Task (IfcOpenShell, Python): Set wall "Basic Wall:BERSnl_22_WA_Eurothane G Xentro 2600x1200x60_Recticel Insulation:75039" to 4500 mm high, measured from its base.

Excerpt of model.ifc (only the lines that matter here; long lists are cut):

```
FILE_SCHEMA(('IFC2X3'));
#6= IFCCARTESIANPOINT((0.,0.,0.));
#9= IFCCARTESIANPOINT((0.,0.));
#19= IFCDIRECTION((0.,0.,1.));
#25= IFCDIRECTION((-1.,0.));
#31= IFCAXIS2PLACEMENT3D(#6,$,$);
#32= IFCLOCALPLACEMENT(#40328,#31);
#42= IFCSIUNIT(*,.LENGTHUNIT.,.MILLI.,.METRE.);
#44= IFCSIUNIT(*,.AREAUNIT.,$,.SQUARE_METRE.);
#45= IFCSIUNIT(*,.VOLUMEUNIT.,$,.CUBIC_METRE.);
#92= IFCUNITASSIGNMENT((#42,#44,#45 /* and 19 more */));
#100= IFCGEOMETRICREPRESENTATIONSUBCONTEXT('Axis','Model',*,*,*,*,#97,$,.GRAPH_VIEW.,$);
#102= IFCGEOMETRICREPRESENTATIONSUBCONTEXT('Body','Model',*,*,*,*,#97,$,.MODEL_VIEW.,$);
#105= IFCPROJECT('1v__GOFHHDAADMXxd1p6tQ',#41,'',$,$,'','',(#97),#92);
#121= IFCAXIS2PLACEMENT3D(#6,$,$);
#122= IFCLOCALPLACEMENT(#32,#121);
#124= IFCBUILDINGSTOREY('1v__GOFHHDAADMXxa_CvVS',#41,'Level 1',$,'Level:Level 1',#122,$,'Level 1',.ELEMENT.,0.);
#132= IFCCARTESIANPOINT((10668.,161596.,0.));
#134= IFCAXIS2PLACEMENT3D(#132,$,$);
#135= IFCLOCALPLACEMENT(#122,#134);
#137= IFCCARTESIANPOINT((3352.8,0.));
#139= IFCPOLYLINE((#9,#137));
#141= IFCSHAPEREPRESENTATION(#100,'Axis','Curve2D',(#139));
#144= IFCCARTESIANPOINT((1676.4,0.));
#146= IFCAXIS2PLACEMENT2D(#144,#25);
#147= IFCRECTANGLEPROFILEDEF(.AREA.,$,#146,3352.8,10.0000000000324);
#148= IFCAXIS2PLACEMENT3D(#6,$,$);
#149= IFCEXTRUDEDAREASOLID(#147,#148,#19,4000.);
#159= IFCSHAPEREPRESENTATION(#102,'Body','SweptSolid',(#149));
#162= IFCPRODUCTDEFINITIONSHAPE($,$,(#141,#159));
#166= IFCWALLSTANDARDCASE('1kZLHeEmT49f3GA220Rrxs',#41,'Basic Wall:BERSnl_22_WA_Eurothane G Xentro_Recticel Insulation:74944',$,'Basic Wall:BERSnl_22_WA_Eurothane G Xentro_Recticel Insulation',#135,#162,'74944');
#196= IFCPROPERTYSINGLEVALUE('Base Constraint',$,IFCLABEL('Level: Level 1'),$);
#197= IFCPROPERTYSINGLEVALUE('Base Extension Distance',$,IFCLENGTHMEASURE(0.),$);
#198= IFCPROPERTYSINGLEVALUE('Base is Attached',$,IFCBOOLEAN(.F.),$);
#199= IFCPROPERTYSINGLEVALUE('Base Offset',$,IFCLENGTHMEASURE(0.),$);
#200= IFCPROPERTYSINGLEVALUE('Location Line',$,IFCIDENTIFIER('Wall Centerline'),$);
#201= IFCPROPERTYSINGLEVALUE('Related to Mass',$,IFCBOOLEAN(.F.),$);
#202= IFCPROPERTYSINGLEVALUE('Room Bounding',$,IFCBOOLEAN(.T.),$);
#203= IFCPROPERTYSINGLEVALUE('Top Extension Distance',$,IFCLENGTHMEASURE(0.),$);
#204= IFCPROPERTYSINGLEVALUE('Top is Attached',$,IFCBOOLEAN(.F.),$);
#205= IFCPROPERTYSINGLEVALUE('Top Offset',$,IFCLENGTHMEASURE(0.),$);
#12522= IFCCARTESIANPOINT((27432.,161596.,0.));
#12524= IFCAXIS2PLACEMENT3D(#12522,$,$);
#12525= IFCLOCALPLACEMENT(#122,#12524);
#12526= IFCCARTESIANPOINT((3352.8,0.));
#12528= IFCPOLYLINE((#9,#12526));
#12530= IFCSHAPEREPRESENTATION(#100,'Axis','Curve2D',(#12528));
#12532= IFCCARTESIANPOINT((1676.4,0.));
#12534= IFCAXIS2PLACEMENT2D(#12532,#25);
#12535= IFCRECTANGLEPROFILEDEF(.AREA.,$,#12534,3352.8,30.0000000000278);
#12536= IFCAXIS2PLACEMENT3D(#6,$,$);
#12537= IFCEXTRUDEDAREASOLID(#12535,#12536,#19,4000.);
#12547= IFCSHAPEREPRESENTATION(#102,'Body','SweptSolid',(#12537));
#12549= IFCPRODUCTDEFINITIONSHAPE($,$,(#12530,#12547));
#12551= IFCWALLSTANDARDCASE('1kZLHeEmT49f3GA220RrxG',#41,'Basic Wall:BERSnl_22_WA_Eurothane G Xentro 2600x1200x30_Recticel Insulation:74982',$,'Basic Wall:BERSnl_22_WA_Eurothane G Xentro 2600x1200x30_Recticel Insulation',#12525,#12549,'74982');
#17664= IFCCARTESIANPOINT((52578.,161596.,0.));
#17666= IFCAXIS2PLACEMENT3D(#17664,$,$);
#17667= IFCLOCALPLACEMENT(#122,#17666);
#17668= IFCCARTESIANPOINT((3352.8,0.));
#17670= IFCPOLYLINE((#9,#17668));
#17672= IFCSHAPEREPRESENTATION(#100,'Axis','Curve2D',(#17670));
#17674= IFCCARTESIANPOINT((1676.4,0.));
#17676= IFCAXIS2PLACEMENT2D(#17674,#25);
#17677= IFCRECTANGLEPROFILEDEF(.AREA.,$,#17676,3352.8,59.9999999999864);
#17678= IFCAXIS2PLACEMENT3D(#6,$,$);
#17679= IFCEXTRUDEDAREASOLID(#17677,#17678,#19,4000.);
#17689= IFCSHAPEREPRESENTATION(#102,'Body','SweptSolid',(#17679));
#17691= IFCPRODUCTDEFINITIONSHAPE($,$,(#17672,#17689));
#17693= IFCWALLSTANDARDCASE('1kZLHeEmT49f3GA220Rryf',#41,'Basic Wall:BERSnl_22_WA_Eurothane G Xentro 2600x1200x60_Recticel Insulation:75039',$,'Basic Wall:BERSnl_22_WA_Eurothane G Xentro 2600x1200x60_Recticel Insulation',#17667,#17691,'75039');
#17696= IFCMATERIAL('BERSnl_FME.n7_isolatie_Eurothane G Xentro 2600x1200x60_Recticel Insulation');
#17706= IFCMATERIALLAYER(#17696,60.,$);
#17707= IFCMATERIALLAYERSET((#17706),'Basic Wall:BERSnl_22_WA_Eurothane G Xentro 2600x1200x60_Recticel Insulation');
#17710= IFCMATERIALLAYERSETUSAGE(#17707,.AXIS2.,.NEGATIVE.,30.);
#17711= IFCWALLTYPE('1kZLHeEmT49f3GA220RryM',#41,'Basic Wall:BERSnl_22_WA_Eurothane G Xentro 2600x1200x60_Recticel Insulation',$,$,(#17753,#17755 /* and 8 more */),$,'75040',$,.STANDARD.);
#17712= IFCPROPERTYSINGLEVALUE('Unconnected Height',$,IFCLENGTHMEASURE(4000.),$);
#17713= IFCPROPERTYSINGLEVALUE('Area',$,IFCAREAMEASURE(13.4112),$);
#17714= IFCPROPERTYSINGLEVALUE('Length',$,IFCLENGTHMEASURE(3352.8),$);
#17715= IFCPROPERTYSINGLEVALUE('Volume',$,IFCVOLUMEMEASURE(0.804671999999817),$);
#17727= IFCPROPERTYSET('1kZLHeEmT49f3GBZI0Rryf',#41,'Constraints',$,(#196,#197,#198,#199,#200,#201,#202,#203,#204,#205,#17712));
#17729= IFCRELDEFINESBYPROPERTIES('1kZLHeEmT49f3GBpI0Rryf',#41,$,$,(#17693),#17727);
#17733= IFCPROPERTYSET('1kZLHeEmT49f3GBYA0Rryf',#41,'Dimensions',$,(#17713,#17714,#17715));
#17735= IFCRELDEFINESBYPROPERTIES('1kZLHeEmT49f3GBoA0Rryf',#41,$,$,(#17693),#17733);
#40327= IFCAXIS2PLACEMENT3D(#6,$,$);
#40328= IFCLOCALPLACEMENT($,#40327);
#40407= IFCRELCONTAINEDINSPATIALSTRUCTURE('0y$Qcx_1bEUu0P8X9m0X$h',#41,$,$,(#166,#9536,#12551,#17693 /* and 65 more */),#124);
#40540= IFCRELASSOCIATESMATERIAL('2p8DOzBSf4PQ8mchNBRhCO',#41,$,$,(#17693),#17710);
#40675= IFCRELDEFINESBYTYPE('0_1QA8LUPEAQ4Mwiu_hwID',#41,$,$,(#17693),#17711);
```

```python
import ifcopenshell
import ifcopenshell.api.pset
import ifcopenshell.geom
import ifcopenshell.util.element
import ifcopenshell.util.representation
import ifcopenshell.util.shape
import ifcopenshell.util.unit

model = ifcopenshell.open("model.ifc")
unit_scale = ifcopenshell.util.unit.calculate_unit_scale(model)
area_scale = ifcopenshell.util.unit.calculate_unit_scale(model, "AREAUNIT")
volume_scale = ifcopenshell.util.unit.calculate_unit_scale(model, "VOLUMEUNIT")
settings = ifcopenshell.geom.settings()


def volume(element):
    """Net volume in cubic metres, openings subtracted."""
    shape = ifcopenshell.geom.create_shape(settings, element)
    return ifcopenshell.util.shape.get_volume(shape.geometry)


wall = model.by_guid("1kZLHeEmT49f3GA220Rryf")
before = volume(wall)

body = ifcopenshell.util.representation.get_representation(wall, "Model", "Body")
solid = body.Items[0]
old_height = solid.Depth
solid.Depth = 4.5 / unit_scale
after = volume(wall)
thickness = 0.06  # wall thickness in metres

# Update the stored height, areas and volumes.
pset = model.by_id(ifcopenshell.util.element.get_pset(wall, "Constraints", should_inherit=False)["id"])
ifcopenshell.api.pset.edit_pset(model, pset=pset, properties={
    "Unconnected Height": model.create_entity("IfcLengthMeasure", solid.Depth),
})
pset = model.by_id(ifcopenshell.util.element.get_pset(wall, "Dimensions", should_inherit=False)["id"])
ifcopenshell.api.pset.edit_pset(model, pset=pset, properties={
    "Area": model.create_entity("IfcAreaMeasure", after / thickness / area_scale),
    "Volume": model.create_entity("IfcVolumeMeasure", after / volume_scale),
})

print(f"height {old_height:g} -> {solid.Depth:g}, volume {before:.3f} -> {after:.3f} m3")

model.write("model_edited.ifc")
```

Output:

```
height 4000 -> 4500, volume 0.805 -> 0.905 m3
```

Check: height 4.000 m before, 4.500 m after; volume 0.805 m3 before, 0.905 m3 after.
